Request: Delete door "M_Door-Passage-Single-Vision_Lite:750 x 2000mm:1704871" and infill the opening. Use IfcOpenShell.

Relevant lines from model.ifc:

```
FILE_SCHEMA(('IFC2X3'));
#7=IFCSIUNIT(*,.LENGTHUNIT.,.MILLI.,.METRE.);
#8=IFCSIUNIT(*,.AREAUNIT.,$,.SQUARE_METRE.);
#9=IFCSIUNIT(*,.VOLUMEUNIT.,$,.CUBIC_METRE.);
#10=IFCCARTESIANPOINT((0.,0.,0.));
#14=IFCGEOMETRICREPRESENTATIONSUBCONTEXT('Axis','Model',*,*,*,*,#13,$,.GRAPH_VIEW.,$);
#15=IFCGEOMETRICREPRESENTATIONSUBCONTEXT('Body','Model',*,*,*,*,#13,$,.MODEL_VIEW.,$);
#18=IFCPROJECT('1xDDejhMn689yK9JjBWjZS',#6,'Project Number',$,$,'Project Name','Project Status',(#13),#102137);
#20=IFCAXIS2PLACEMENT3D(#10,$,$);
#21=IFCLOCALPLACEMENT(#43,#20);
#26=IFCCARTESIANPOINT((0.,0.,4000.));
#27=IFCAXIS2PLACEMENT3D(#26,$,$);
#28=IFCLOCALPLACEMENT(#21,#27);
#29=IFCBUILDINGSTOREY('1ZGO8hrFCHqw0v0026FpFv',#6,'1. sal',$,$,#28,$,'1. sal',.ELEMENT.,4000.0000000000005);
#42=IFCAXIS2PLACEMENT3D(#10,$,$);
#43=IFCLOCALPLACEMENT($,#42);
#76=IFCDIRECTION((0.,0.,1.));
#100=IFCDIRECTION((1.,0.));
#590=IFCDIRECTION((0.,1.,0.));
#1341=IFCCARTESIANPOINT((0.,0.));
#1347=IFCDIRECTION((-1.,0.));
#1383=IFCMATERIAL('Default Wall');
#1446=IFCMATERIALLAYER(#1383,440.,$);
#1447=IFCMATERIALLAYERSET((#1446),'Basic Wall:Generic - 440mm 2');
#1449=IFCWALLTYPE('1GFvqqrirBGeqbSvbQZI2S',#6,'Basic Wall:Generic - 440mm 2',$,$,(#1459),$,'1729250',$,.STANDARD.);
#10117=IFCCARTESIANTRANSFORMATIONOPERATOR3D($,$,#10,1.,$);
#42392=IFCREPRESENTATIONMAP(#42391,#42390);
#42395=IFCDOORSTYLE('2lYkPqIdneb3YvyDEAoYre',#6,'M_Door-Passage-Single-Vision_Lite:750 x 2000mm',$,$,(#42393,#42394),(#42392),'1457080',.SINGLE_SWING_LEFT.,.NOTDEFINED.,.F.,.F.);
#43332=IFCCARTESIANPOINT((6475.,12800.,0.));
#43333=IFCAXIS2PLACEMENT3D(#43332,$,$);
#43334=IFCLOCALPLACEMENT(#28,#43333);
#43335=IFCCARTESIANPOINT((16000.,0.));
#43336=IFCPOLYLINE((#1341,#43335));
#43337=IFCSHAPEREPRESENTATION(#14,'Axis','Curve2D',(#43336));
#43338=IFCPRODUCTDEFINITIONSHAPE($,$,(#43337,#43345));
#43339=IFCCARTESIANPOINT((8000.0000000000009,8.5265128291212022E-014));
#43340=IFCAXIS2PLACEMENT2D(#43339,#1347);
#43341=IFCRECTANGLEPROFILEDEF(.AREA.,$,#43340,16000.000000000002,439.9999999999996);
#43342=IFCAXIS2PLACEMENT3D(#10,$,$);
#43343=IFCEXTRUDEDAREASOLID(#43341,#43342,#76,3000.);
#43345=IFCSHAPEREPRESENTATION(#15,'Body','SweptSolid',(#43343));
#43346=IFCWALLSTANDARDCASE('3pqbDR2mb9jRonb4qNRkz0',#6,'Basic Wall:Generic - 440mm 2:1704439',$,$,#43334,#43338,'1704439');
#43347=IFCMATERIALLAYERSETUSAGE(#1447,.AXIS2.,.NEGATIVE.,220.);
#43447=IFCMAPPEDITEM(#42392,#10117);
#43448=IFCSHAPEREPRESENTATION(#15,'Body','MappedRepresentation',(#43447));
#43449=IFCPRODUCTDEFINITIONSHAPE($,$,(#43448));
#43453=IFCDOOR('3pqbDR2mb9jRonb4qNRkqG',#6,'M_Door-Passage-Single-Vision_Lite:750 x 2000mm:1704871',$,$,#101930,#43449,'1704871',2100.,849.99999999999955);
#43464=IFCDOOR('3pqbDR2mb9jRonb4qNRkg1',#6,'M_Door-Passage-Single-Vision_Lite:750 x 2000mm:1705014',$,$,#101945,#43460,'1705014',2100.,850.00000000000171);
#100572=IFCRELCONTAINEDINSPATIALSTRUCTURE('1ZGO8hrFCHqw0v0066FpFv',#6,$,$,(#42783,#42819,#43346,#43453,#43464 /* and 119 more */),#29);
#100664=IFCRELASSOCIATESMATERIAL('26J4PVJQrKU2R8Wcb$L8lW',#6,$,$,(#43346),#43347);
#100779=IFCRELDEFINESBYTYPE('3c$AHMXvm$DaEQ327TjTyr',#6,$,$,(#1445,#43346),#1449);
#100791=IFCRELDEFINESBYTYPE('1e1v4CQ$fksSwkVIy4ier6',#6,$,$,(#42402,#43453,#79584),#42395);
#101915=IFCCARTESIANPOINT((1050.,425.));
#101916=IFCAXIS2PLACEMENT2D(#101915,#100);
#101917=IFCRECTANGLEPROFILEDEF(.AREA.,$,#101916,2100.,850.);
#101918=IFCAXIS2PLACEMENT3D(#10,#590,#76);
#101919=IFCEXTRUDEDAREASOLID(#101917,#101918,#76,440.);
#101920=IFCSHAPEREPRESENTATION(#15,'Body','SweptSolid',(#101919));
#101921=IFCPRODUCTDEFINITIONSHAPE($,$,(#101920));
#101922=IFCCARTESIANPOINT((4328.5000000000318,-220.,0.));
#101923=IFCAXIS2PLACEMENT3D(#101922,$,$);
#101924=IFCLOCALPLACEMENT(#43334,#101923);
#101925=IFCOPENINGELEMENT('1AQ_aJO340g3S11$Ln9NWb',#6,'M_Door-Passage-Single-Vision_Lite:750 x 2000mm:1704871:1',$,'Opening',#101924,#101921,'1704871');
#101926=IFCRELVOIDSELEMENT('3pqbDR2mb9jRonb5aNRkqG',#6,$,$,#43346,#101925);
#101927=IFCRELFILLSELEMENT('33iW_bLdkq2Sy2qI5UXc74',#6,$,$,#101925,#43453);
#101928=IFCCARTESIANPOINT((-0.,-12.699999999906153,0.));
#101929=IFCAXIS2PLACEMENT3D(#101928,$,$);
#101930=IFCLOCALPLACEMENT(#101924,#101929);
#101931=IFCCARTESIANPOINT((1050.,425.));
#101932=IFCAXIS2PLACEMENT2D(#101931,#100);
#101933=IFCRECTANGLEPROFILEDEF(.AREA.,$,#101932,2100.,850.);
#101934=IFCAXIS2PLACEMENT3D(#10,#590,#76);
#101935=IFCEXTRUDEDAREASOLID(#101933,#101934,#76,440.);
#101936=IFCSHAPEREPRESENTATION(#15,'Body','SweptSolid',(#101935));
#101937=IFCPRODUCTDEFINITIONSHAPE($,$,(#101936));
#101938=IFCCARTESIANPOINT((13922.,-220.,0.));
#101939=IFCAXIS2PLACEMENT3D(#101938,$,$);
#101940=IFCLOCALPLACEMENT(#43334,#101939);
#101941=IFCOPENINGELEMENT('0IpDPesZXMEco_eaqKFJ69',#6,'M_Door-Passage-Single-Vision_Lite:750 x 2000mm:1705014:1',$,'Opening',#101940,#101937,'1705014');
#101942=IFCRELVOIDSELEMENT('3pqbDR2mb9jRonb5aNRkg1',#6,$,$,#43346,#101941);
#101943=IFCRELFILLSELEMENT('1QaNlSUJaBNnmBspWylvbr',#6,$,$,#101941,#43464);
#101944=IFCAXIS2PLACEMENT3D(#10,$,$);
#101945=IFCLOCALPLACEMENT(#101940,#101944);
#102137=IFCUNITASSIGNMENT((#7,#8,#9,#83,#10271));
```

```python
import ifcopenshell
import ifcopenshell.api.feature
import ifcopenshell.api.root
import ifcopenshell.geom
import ifcopenshell.util.shape

model = ifcopenshell.open("model.ifc")
settings = ifcopenshell.geom.settings()


def volume(element):
    """Net volume in cubic metres, openings subtracted."""
    shape = ifcopenshell.geom.create_shape(settings, element)
    return ifcopenshell.util.shape.get_volume(shape.geometry)


door = model.by_guid("3pqbDR2mb9jRonb4qNRkqG")
opening = door.FillsVoids[0].RelatingOpeningElement
wall = opening.VoidsElements[0].RelatingBuildingElement
before = volume(wall)

ifcopenshell.api.root.remove_product(model, product=door)
ifcopenshell.api.feature.remove_feature(model, feature=opening)

after = volume(wall)

print(f"wall volume {before:.3f} -> {after:.3f} m3")

model.write("model_rev.ifc")
```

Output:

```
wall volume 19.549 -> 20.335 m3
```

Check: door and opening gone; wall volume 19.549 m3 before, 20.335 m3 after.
